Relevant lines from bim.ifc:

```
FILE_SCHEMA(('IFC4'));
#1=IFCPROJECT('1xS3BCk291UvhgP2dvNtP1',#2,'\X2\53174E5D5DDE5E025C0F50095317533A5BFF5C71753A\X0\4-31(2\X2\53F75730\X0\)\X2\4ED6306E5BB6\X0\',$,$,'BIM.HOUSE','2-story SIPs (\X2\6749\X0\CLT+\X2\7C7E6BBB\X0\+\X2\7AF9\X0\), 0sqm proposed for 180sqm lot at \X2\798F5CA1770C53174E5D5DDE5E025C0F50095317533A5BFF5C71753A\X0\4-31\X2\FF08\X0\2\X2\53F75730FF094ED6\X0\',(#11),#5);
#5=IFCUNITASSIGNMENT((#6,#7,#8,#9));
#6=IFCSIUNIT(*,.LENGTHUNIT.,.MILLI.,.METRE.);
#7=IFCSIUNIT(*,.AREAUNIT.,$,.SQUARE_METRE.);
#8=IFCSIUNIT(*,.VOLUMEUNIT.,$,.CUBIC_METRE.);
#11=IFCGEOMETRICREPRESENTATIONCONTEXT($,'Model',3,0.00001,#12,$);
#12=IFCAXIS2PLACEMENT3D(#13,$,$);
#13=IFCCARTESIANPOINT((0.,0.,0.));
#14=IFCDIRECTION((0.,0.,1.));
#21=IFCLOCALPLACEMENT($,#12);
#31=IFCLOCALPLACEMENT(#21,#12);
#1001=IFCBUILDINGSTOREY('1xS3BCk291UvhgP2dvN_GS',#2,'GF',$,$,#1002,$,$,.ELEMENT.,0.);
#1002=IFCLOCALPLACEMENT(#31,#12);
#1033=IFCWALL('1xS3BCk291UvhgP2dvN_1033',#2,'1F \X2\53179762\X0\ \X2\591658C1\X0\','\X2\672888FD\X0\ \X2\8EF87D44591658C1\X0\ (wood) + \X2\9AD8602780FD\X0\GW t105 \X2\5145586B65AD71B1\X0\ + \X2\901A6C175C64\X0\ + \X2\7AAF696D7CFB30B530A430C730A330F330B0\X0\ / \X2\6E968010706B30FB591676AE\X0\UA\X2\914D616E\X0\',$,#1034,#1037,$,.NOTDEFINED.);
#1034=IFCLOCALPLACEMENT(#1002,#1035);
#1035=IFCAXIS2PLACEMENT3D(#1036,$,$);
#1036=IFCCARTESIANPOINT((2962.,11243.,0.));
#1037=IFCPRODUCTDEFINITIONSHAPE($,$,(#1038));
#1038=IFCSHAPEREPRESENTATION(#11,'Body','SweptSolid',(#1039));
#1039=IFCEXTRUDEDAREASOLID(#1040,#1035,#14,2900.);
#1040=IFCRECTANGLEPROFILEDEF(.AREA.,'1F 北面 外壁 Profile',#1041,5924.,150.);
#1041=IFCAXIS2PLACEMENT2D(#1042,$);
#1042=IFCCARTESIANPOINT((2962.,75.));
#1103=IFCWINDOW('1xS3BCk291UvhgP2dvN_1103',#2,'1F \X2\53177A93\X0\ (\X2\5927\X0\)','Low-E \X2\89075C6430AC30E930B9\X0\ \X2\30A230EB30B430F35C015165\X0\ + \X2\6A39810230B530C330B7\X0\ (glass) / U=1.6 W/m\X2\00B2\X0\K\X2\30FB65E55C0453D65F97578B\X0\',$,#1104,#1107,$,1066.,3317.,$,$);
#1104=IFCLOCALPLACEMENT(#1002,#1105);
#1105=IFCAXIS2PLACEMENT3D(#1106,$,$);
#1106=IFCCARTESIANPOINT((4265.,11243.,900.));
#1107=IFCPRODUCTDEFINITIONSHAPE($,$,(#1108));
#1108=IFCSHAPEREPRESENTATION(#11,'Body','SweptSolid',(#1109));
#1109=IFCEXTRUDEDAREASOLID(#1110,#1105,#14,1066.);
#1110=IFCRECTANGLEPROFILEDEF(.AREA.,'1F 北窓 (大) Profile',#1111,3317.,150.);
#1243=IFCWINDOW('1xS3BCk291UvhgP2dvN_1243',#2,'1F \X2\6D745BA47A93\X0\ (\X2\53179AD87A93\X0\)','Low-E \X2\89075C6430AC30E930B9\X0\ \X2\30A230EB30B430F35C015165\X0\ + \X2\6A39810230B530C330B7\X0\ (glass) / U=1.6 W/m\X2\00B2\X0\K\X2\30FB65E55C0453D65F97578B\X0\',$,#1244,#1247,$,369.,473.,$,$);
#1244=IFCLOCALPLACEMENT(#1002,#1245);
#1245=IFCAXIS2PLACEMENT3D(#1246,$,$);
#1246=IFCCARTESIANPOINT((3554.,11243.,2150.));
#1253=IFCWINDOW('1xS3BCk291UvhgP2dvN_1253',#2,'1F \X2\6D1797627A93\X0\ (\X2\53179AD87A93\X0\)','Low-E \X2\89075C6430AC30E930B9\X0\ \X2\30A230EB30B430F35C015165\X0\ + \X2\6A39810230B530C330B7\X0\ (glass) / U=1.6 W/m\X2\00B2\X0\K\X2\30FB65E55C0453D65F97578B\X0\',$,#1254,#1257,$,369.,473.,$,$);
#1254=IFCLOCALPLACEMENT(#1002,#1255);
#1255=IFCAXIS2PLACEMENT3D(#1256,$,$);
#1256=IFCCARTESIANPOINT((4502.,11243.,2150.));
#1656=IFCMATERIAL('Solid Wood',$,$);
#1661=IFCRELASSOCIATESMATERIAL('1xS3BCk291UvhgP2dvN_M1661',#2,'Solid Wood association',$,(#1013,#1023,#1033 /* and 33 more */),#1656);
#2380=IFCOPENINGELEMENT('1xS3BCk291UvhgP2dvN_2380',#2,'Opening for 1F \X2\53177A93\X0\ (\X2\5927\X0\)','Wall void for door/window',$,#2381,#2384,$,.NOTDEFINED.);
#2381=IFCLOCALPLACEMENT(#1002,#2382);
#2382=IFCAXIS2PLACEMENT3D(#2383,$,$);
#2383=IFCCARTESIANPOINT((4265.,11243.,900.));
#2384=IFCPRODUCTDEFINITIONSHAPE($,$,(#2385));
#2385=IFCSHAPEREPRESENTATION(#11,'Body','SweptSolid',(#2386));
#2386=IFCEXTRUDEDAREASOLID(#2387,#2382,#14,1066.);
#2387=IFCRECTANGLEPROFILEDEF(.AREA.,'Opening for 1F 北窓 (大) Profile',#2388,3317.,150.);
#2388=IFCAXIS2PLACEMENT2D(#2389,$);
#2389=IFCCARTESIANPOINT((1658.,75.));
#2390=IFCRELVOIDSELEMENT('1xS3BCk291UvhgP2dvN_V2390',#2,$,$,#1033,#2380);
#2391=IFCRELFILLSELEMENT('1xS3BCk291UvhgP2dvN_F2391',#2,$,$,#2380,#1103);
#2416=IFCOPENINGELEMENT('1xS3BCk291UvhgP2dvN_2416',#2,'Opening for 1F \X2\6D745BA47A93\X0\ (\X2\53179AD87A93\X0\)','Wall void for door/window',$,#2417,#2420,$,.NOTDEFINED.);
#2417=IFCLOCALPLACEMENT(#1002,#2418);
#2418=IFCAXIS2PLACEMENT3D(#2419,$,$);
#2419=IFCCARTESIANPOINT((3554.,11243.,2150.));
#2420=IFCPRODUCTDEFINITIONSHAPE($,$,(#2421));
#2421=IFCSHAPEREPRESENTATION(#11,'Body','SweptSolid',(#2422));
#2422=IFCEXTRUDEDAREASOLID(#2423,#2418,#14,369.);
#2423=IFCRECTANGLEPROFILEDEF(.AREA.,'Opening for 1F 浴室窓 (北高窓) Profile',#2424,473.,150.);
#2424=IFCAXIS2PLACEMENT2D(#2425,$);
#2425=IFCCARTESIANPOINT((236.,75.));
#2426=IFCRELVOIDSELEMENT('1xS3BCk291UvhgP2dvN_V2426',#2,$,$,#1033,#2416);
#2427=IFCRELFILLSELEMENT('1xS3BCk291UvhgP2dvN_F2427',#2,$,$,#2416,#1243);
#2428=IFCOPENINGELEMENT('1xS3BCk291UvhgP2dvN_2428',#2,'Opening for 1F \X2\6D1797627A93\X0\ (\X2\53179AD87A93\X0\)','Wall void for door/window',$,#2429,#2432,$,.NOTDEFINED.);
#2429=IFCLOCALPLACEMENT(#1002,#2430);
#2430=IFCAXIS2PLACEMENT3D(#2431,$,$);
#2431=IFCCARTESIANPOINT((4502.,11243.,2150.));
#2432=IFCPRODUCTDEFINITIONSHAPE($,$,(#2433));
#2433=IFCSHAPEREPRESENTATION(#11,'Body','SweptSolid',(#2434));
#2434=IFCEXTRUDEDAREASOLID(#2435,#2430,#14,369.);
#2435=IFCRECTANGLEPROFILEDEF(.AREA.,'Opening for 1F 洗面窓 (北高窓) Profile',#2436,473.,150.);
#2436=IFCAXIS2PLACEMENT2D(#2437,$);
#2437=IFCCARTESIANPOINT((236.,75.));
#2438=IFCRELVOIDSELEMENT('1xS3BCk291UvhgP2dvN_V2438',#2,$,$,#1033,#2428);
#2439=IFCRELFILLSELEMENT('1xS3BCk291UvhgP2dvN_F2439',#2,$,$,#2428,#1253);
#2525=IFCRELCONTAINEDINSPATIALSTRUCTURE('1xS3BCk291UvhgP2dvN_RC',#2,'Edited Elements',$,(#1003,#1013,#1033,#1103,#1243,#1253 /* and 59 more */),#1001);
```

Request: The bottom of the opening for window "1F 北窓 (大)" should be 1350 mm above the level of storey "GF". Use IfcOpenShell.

```python
import numpy as np
import ifcopenshell
import ifcopenshell.api.geometry
import ifcopenshell.geom
import ifcopenshell.util.element
import ifcopenshell.util.placement
import ifcopenshell.util.shape
import ifcopenshell.util.unit

model = ifcopenshell.open("bim.ifc")
unit_scale = ifcopenshell.util.unit.calculate_unit_scale(model)

window = model.by_guid("1xS3BCk291UvhgP2dvN_1103")
opening = window.FillsVoids[0].RelatingOpeningElement
storey = ifcopenshell.util.element.get_container(window, ifc_class="IfcBuildingStorey")
level = ifcopenshell.util.placement.get_local_placement(storey.ObjectPlacement)[2, 3]

# The opening's origin need not be at the sill, so measure its lowest point.
shape = ifcopenshell.geom.create_shape(ifcopenshell.geom.settings(), opening)
bottom = ifcopenshell.util.shape.get_shape_bottom_elevation(shape, shape.geometry) / unit_scale
dz = level + 1350.0 - bottom

shift = np.array([0.0, 0.0, dz])
# The window is not placed relative to its opening, so move both.
for product in (opening, window):
    matrix = ifcopenshell.util.placement.get_local_placement(product.ObjectPlacement)
    matrix[:3, 3] += shift
    ifcopenshell.api.geometry.edit_object_placement(model, product=product, matrix=matrix, is_si=False)

print(f"moved by {dz * unit_scale:+.3f} m")

model.write("bim_v2.ifc")
```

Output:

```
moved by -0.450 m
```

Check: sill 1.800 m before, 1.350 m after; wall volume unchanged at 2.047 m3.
